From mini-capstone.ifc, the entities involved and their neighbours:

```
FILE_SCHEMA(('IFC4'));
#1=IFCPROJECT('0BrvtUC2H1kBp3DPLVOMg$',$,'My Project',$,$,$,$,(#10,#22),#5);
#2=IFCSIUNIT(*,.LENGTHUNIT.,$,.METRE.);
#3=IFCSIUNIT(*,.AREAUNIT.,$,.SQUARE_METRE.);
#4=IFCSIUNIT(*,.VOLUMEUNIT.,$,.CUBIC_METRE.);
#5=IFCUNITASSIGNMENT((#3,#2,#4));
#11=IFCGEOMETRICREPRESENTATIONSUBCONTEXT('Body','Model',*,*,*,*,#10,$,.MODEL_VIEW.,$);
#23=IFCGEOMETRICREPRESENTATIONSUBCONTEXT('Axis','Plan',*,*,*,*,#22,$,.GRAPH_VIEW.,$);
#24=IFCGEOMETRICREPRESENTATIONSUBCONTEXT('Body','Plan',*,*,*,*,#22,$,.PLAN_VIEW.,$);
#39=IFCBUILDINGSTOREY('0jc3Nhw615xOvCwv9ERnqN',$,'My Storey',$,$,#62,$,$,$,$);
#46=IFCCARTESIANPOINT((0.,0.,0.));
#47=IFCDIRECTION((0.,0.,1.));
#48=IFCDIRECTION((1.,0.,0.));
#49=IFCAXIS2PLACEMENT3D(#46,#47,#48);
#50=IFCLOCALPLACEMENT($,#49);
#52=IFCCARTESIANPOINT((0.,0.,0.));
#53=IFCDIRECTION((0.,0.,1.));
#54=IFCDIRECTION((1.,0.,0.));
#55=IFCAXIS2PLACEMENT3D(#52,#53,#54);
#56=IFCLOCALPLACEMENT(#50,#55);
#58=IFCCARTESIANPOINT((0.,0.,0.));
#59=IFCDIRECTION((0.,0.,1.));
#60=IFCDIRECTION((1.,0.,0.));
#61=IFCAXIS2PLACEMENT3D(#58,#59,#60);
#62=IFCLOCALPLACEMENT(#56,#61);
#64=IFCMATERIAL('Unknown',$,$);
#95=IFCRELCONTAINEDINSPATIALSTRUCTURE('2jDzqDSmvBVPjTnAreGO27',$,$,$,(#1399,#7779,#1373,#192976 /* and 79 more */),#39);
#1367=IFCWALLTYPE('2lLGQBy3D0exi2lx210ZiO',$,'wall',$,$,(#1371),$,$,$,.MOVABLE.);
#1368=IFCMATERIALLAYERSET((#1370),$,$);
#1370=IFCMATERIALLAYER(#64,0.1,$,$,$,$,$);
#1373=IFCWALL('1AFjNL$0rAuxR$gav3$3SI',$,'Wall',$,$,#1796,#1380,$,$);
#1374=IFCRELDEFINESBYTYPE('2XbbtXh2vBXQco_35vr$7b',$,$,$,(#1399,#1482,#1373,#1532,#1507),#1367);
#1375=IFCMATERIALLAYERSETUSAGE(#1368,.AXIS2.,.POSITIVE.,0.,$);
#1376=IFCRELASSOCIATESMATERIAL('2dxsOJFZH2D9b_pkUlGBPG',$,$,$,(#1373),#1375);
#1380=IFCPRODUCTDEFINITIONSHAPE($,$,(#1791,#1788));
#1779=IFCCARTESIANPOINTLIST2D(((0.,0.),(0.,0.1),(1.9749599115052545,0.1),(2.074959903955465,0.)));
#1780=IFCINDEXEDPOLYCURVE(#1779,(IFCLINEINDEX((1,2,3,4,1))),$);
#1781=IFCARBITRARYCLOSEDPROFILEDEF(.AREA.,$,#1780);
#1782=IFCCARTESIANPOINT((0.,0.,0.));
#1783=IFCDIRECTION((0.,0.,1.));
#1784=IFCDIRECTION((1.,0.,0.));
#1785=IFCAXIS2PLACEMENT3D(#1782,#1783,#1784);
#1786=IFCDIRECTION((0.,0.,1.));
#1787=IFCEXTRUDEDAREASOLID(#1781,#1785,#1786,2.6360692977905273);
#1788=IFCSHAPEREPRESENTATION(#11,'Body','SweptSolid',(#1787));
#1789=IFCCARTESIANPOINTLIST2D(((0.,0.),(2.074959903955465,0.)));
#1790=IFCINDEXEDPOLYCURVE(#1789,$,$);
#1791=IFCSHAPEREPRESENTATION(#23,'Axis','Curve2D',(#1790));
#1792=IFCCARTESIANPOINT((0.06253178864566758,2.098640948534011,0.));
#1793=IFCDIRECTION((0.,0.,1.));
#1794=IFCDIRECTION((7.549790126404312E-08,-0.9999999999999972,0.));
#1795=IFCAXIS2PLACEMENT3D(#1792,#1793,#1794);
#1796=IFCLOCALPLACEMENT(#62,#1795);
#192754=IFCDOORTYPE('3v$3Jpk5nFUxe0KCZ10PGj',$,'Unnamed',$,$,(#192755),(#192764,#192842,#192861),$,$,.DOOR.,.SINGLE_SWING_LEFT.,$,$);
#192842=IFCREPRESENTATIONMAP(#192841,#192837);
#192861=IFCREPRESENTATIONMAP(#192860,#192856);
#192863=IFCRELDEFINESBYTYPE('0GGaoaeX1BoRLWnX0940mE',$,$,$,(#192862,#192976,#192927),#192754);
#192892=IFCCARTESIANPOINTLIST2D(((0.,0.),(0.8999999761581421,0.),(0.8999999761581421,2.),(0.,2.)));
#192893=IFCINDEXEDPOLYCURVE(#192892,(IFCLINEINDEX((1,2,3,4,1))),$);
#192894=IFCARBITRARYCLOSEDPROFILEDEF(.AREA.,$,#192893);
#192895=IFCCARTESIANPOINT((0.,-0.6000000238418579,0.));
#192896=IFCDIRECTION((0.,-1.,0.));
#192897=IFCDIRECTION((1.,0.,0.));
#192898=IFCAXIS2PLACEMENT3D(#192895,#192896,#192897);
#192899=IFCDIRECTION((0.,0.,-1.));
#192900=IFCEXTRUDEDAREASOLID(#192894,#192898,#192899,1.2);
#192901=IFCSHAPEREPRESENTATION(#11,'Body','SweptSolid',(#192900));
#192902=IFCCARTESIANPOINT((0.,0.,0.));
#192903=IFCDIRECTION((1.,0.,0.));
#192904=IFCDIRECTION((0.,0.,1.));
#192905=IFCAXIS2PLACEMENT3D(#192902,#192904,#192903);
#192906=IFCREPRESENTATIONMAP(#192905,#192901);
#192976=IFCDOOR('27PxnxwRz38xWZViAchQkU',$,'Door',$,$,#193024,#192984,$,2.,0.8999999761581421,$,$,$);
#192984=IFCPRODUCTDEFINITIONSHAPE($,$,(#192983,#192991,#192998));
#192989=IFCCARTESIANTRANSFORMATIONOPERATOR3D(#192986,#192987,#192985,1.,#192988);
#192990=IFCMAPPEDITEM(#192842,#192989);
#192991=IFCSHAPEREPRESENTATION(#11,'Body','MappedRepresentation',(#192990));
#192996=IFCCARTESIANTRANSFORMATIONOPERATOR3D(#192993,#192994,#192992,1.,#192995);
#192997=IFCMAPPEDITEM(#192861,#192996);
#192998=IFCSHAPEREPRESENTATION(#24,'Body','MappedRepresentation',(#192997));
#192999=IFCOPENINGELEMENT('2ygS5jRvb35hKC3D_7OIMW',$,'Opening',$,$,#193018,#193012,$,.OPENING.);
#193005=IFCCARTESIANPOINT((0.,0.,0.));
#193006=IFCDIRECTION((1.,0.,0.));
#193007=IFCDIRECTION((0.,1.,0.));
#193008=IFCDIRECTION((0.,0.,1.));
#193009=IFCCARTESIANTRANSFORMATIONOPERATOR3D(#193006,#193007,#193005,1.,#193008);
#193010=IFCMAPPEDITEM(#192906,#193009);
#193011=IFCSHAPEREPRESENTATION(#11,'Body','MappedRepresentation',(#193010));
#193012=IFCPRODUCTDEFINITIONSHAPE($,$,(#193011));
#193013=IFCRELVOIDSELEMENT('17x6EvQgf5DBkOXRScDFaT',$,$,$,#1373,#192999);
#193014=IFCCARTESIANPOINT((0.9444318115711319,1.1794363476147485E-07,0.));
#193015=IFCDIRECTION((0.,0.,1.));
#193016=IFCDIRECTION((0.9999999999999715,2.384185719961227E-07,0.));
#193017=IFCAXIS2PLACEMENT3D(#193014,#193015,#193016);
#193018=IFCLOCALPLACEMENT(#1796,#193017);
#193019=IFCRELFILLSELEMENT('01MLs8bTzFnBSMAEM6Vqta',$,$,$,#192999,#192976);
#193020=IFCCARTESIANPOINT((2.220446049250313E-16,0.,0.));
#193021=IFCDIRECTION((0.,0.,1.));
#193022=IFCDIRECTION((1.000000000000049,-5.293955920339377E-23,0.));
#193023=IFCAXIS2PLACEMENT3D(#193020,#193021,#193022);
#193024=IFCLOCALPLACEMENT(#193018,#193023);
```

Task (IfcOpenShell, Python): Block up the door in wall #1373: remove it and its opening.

```python
import ifcopenshell
import ifcopenshell.api.feature
import ifcopenshell.api.root
import ifcopenshell.geom
import ifcopenshell.util.shape

model = ifcopenshell.open("mini-capstone.ifc")
settings = ifcopenshell.geom.settings()


def volume(element):
    """Net volume in cubic metres, openings subtracted."""
    shape = ifcopenshell.geom.create_shape(settings, element)
    return ifcopenshell.util.shape.get_volume(shape.geometry)


door = model.by_guid("27PxnxwRz38xWZViAchQkU")
opening = door.FillsVoids[0].RelatingOpeningElement
wall = opening.VoidsElements[0].RelatingBuildingElement
before = volume(wall)

ifcopenshell.api.root.remove_product(model, product=door)
ifcopenshell.api.feature.remove_feature(model, feature=opening)

after = volume(wall)

print(f"wall volume {before:.3f} -> {after:.3f} m3")

model.write("mini-capstone_updated.ifc")
```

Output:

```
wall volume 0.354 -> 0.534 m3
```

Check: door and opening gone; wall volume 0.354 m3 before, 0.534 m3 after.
